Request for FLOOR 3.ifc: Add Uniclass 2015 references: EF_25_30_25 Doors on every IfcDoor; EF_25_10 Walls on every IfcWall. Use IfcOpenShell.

First a look at what the model holds.

```python
import ifcopenshell

model = ifcopenshell.open("FLOOR 3.ifc")
print(model.schema)
print("classifications:", [c.Name for c in model.by_type("IfcClassification")])
for ifc_class in ("IfcDoor", "IfcRoof", "IfcStair", "IfcWall", "IfcWindow"):
    print(ifc_class, len(model.by_type(ifc_class)))
```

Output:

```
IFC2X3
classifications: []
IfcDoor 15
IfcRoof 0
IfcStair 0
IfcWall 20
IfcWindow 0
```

```python
import ifcopenshell
import ifcopenshell.api.classification

model = ifcopenshell.open("FLOOR 3.ifc")

# IFC2X3 requires Source and Edition and has no link from the project to the system.
system = model.create_entity("IfcClassification", Source="NBS", Edition="2015", Name="Uniclass 2015")

codes = {
    "IfcDoor": ("EF_25_30_25", "Doors"),
    "IfcWall": ("EF_25_10", "Walls"),
}
for ifc_class, (code, name) in codes.items():
    products = model.by_type(ifc_class)
    ifcopenshell.api.classification.add_reference(
        model, products=products, classification=system, identification=code, name=name
    )
    print(code, len(products))

model.write("FLOOR 3_v2.ifc")
```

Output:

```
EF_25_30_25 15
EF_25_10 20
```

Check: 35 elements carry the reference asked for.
